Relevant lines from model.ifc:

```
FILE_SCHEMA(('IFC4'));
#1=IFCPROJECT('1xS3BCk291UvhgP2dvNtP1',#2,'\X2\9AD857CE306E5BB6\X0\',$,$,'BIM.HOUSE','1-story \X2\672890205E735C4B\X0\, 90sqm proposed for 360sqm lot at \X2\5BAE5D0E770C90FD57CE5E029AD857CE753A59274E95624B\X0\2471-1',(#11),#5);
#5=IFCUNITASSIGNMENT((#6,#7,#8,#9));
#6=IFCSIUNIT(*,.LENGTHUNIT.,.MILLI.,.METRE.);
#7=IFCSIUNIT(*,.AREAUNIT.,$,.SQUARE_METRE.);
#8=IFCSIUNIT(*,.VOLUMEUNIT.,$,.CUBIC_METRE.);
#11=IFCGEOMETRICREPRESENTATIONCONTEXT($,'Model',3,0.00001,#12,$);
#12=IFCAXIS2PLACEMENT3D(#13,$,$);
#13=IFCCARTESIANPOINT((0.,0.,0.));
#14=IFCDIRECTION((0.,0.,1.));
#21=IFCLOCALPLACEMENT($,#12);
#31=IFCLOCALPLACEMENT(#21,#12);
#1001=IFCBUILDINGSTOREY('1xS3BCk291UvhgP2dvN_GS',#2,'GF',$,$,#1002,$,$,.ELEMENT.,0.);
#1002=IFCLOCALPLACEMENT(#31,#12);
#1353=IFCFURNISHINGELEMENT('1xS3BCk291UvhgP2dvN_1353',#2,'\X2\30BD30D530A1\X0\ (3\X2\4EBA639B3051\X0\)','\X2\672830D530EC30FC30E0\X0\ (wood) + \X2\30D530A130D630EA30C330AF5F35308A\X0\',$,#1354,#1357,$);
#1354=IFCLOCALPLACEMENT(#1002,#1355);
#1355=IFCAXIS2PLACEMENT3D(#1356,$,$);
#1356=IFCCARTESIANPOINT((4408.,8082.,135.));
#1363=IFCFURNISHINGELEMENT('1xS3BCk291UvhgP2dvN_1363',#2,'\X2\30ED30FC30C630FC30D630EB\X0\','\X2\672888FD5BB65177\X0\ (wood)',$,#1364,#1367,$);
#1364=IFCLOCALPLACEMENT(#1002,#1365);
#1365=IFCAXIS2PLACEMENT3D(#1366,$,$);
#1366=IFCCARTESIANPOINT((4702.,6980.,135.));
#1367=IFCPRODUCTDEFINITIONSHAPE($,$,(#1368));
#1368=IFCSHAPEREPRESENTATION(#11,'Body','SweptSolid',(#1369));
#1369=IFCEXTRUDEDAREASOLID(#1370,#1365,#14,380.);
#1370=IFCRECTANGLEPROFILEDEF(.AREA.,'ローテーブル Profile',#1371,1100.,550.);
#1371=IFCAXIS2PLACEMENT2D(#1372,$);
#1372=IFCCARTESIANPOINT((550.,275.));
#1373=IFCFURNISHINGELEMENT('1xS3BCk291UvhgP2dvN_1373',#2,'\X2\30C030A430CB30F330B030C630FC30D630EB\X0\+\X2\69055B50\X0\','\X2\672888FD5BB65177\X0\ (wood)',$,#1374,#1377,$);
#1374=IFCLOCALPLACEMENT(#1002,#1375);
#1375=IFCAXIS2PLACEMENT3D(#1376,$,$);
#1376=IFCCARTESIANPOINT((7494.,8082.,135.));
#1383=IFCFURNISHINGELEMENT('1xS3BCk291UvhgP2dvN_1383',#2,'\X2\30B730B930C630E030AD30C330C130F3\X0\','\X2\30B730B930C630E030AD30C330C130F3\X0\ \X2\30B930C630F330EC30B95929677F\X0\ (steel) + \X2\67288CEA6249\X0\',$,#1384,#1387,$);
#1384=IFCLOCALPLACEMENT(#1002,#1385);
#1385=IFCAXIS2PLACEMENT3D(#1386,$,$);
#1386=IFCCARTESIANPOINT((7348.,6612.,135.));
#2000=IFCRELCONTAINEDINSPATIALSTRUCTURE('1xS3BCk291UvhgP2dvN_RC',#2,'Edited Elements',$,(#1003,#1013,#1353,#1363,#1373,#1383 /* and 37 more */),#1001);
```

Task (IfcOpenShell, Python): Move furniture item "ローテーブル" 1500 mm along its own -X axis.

```python
import ifcopenshell
import ifcopenshell.api.geometry
import ifcopenshell.util.placement

model = ifcopenshell.open("model.ifc")

item = model.by_id(1363)
matrix = ifcopenshell.util.placement.get_local_placement(item.ObjectPlacement)
matrix[:3, 3] -= matrix[:3, 0] * 1500.0
ifcopenshell.api.geometry.edit_object_placement(model, product=item, matrix=matrix, is_si=False)

print(ifcopenshell.util.placement.get_local_placement(item.ObjectPlacement).round(3) + 0.0)

model.write("model_v2.ifc")
```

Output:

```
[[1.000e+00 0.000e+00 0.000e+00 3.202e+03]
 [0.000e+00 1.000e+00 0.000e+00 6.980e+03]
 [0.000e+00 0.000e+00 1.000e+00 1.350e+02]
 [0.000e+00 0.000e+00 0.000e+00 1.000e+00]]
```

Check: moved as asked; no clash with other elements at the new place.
